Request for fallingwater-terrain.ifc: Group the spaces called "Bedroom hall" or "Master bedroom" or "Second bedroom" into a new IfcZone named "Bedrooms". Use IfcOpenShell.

First a look at what the model holds.

```python
import ifcopenshell

model = ifcopenshell.open("fallingwater-terrain.ifc")
print(model.schema)
seen = {}
for space in model.by_type("IfcSpace"):
    seen[space.LongName] = seen.get(space.LongName, 0) + 1
for name, count in sorted(seen.items(), key=str):
    print(count, "x", name)
print("zones:", [z.Name for z in model.by_type("IfcZone")][:20])
```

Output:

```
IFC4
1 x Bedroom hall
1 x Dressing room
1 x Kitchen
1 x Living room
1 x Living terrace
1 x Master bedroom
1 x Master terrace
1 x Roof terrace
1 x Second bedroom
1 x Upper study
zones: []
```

```python
import ifcopenshell
import ifcopenshell.api.group
import ifcopenshell.api.root

model = ifcopenshell.open("fallingwater-terrain.ifc")

names = {"Bedroom hall", "Master bedroom", "Second bedroom"}
spaces = [s for s in model.by_type("IfcSpace") if s.LongName in names]

zone = ifcopenshell.api.root.create_entity(model, ifc_class="IfcZone", name="Bedrooms")
ifcopenshell.api.group.assign_group(model, products=spaces, group=zone)
print(len(spaces), "spaces in", zone.Name)

model.write("fallingwater-terrain_edited.ifc")
```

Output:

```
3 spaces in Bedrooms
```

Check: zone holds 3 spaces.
